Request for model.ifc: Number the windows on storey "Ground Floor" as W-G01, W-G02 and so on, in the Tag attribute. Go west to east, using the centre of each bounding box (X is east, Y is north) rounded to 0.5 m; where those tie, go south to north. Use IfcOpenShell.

First a look at what the model holds.

```python
import ifcopenshell
import ifcopenshell.util.element
import ifcopenshell.util.placement

model = ifcopenshell.open("model.ifc")
print(model.schema)
storey = next(s for s in model.by_type("IfcBuildingStorey") if s.Name == "Ground Floor")
windows = [e for e in ifcopenshell.util.element.get_decomposition(storey) if e.is_a("IfcWindow")]
for e in sorted(windows, key=lambda e: e.id()):
    origin = ifcopenshell.util.placement.get_local_placement(e.ObjectPlacement)[:3, 3]
    print(e.id(), e.Tag, e.Name, origin.round(2) + 0.0, sep=" | ")
```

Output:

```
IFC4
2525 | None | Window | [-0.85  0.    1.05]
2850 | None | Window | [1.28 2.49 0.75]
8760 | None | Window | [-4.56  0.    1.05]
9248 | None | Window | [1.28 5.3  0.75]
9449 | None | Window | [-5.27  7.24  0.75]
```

```python
import ifcopenshell
import ifcopenshell.geom
import ifcopenshell.util.element
import ifcopenshell.util.shape

model = ifcopenshell.open("model.ifc")
settings = ifcopenshell.geom.settings()
settings.set("use-world-coords", True)


def centre(element):
    shape = ifcopenshell.geom.create_shape(settings, element)
    return ifcopenshell.util.shape.get_bbox_centroid(shape.geometry)


storey = next(s for s in model.by_type("IfcBuildingStorey") if s.Name == "Ground Floor")
windows = [e for e in ifcopenshell.util.element.get_decomposition(storey) if e.is_a("IfcWindow")]

# Insertion points can sit at a corner or the storey origin, so sort by the geometry (in metres).
centres = {e: centre(e) for e in windows}
windows.sort(key=lambda e: (round(centres[e][0] / 0.5), centres[e][1]))

for i, e in enumerate(windows, start=1):
    number = f"W-G{i:02d}"
    e.Tag = number
    print(e.id(), number)

model.write("model_edited.ifc")
```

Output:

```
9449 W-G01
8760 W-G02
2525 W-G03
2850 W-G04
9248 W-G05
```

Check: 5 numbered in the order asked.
